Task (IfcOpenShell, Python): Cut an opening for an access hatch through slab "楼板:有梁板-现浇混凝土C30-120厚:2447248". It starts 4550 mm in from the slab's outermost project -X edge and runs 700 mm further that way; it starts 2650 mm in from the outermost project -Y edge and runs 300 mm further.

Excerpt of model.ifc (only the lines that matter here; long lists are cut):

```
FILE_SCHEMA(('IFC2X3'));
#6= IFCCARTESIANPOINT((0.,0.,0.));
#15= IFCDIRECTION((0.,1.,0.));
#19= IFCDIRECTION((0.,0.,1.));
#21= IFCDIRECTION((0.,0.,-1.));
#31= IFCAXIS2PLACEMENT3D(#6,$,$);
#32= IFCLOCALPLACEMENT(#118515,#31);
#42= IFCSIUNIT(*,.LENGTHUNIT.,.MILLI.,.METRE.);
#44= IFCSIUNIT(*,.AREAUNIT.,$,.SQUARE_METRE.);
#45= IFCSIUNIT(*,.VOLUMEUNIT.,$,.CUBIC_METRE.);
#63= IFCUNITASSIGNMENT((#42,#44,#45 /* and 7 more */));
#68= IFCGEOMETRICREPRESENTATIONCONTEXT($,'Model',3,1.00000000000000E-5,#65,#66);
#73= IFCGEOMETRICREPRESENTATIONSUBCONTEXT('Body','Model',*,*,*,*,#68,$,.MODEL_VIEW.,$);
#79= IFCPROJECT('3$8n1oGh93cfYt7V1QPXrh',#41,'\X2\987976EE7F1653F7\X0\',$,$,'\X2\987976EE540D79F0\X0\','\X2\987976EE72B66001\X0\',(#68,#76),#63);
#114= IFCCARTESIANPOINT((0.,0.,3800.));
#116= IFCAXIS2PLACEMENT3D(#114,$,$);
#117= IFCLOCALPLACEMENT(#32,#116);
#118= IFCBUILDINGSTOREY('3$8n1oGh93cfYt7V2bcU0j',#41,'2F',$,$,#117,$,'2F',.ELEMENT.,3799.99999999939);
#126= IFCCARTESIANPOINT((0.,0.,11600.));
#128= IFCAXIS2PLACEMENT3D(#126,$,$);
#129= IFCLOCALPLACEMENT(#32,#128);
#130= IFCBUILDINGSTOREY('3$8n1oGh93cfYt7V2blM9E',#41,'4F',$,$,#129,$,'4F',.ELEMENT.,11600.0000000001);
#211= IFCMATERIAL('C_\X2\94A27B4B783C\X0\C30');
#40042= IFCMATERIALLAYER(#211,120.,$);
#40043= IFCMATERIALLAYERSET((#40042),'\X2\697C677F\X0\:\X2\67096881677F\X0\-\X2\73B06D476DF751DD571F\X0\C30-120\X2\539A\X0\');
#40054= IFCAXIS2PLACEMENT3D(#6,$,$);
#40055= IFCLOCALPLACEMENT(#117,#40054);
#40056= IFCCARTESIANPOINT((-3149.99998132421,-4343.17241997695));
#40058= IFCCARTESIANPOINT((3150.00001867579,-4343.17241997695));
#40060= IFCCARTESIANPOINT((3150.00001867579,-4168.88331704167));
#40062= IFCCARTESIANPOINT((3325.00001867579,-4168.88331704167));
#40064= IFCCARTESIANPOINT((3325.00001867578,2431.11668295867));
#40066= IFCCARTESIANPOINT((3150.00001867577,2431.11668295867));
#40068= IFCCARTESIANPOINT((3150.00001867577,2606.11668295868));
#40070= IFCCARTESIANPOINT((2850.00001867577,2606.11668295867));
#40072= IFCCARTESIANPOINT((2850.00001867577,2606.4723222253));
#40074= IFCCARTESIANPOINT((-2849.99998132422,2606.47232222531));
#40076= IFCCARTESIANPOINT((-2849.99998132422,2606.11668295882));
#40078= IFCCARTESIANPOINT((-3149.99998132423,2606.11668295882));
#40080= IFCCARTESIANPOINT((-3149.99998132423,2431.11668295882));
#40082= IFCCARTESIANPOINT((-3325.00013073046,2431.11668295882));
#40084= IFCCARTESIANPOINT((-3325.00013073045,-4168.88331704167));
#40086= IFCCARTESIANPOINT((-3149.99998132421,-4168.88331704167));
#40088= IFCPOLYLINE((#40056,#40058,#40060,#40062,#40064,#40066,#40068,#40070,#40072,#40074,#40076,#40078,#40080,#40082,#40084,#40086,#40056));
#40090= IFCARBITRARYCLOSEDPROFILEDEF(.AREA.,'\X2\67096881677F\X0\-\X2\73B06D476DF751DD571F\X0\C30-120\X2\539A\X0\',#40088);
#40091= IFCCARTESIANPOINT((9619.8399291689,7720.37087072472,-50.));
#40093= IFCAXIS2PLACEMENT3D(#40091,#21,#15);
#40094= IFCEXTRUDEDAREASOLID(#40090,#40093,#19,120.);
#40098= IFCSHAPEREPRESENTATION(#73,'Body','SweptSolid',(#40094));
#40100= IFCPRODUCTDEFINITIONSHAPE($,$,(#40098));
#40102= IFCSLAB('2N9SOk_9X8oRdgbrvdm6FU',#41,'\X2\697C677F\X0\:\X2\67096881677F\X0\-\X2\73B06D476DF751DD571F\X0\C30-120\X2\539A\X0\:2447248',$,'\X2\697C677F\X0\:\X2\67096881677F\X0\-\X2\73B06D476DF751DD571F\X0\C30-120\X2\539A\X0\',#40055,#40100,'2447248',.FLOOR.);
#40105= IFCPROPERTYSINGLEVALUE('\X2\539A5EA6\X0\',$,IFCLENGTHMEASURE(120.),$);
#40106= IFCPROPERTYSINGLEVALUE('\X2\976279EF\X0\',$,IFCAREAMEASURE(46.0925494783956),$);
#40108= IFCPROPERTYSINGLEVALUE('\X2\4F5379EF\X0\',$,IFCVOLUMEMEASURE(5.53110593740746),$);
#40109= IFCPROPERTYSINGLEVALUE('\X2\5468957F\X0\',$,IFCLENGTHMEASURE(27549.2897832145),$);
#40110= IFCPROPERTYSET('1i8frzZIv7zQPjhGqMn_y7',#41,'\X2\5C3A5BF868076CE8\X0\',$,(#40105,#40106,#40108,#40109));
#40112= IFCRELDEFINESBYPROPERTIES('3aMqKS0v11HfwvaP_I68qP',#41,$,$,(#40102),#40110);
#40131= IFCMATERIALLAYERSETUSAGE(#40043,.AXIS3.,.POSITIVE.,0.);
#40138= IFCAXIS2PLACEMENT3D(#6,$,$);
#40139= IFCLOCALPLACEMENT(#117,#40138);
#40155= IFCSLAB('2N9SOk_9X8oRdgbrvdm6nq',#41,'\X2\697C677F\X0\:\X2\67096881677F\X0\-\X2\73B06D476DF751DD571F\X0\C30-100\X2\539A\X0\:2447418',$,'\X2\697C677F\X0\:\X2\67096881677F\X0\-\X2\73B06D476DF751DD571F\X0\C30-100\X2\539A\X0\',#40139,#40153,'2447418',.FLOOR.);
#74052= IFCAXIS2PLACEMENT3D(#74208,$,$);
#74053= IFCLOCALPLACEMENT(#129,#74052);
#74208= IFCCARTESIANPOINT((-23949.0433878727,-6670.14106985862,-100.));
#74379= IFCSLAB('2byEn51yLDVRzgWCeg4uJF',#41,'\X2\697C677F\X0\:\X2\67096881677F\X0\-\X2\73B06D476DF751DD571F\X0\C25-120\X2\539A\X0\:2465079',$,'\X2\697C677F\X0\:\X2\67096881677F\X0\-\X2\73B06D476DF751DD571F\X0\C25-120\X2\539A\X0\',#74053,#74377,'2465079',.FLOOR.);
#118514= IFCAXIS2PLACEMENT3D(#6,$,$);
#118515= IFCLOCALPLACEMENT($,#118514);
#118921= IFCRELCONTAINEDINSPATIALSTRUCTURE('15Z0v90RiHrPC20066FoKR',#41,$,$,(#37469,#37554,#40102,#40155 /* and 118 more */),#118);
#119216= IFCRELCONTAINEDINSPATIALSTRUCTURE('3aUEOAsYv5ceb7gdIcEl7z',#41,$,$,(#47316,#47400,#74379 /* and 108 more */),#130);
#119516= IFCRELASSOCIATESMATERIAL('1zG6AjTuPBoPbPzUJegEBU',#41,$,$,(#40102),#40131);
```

```python
import numpy as np
import ifcopenshell
import ifcopenshell.api.feature
import ifcopenshell.api.geometry
import ifcopenshell.api.pset
import ifcopenshell.api.root
import ifcopenshell.geom
import ifcopenshell.util.element
import ifcopenshell.util.placement
import ifcopenshell.util.representation
import ifcopenshell.util.shape
import ifcopenshell.util.unit

model = ifcopenshell.open("model.ifc")
unit_scale = ifcopenshell.util.unit.calculate_unit_scale(model)
area_scale = ifcopenshell.util.unit.calculate_unit_scale(model, "AREAUNIT")
volume_scale = ifcopenshell.util.unit.calculate_unit_scale(model, "VOLUMEUNIT")
settings = ifcopenshell.geom.settings()


def volume(element):
    """Net volume in cubic metres, openings subtracted."""
    shape = ifcopenshell.geom.create_shape(settings, element)
    return ifcopenshell.util.shape.get_volume(shape.geometry)


slab = model.by_guid("2N9SOk_9X8oRdgbrvdm6FU")
before = volume(slab)

# Extent in the slab's own axes, in metres. The edges named are its -X and -Y sides.
slab_shape = ifcopenshell.geom.create_shape(settings, slab)
vertices = ifcopenshell.util.shape.get_vertices(slab_shape.geometry)
x_min, y_min, bottom = vertices.min(axis=0)
top = vertices[:, 2].max()

opening = ifcopenshell.api.root.create_entity(model, ifc_class="IfcOpeningElement", name="Access hatch opening")
context = ifcopenshell.util.representation.get_context(model, "Model", "Body", "MODEL_VIEW")
width, depth = 0.7, 0.3
outline = [(0.0, 0.0), (width, 0.0), (width, depth), (0.0, depth), (0.0, 0.0)]
# Overshoot both faces by 50 mm so the cut is clean.
shape = ifcopenshell.api.geometry.add_slab_representation(
    model, context=context, depth=top - bottom + 0.1, polyline=outline
)
ifcopenshell.api.geometry.assign_representation(model, product=opening, representation=shape)

matrix = ifcopenshell.util.placement.get_local_placement(slab.ObjectPlacement)
matrix[:, 3] = matrix @ np.append(np.array([x_min + 4.55, y_min + 2.65, bottom - 0.05]) / unit_scale, 1.0)
ifcopenshell.api.geometry.edit_object_placement(model, product=opening, matrix=matrix, is_si=False)
ifcopenshell.api.feature.add_feature(model, feature=opening, element=slab)

after = volume(slab)

# Update the slab's stored quantities.
pset = model.by_id(ifcopenshell.util.element.get_pset(slab, "尺寸标注", should_inherit=False)["id"])
ifcopenshell.api.pset.edit_pset(model, pset=pset, properties={
    "面积": model.create_entity("IfcAreaMeasure", after / (top - bottom) / area_scale),
    "体积": model.create_entity("IfcVolumeMeasure", after / volume_scale),
})

print(f"slab volume {before:.3f} -> {after:.3f} m3")

model.write("model_v2.ifc")
```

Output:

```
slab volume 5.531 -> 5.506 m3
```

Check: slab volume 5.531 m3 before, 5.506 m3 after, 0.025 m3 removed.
